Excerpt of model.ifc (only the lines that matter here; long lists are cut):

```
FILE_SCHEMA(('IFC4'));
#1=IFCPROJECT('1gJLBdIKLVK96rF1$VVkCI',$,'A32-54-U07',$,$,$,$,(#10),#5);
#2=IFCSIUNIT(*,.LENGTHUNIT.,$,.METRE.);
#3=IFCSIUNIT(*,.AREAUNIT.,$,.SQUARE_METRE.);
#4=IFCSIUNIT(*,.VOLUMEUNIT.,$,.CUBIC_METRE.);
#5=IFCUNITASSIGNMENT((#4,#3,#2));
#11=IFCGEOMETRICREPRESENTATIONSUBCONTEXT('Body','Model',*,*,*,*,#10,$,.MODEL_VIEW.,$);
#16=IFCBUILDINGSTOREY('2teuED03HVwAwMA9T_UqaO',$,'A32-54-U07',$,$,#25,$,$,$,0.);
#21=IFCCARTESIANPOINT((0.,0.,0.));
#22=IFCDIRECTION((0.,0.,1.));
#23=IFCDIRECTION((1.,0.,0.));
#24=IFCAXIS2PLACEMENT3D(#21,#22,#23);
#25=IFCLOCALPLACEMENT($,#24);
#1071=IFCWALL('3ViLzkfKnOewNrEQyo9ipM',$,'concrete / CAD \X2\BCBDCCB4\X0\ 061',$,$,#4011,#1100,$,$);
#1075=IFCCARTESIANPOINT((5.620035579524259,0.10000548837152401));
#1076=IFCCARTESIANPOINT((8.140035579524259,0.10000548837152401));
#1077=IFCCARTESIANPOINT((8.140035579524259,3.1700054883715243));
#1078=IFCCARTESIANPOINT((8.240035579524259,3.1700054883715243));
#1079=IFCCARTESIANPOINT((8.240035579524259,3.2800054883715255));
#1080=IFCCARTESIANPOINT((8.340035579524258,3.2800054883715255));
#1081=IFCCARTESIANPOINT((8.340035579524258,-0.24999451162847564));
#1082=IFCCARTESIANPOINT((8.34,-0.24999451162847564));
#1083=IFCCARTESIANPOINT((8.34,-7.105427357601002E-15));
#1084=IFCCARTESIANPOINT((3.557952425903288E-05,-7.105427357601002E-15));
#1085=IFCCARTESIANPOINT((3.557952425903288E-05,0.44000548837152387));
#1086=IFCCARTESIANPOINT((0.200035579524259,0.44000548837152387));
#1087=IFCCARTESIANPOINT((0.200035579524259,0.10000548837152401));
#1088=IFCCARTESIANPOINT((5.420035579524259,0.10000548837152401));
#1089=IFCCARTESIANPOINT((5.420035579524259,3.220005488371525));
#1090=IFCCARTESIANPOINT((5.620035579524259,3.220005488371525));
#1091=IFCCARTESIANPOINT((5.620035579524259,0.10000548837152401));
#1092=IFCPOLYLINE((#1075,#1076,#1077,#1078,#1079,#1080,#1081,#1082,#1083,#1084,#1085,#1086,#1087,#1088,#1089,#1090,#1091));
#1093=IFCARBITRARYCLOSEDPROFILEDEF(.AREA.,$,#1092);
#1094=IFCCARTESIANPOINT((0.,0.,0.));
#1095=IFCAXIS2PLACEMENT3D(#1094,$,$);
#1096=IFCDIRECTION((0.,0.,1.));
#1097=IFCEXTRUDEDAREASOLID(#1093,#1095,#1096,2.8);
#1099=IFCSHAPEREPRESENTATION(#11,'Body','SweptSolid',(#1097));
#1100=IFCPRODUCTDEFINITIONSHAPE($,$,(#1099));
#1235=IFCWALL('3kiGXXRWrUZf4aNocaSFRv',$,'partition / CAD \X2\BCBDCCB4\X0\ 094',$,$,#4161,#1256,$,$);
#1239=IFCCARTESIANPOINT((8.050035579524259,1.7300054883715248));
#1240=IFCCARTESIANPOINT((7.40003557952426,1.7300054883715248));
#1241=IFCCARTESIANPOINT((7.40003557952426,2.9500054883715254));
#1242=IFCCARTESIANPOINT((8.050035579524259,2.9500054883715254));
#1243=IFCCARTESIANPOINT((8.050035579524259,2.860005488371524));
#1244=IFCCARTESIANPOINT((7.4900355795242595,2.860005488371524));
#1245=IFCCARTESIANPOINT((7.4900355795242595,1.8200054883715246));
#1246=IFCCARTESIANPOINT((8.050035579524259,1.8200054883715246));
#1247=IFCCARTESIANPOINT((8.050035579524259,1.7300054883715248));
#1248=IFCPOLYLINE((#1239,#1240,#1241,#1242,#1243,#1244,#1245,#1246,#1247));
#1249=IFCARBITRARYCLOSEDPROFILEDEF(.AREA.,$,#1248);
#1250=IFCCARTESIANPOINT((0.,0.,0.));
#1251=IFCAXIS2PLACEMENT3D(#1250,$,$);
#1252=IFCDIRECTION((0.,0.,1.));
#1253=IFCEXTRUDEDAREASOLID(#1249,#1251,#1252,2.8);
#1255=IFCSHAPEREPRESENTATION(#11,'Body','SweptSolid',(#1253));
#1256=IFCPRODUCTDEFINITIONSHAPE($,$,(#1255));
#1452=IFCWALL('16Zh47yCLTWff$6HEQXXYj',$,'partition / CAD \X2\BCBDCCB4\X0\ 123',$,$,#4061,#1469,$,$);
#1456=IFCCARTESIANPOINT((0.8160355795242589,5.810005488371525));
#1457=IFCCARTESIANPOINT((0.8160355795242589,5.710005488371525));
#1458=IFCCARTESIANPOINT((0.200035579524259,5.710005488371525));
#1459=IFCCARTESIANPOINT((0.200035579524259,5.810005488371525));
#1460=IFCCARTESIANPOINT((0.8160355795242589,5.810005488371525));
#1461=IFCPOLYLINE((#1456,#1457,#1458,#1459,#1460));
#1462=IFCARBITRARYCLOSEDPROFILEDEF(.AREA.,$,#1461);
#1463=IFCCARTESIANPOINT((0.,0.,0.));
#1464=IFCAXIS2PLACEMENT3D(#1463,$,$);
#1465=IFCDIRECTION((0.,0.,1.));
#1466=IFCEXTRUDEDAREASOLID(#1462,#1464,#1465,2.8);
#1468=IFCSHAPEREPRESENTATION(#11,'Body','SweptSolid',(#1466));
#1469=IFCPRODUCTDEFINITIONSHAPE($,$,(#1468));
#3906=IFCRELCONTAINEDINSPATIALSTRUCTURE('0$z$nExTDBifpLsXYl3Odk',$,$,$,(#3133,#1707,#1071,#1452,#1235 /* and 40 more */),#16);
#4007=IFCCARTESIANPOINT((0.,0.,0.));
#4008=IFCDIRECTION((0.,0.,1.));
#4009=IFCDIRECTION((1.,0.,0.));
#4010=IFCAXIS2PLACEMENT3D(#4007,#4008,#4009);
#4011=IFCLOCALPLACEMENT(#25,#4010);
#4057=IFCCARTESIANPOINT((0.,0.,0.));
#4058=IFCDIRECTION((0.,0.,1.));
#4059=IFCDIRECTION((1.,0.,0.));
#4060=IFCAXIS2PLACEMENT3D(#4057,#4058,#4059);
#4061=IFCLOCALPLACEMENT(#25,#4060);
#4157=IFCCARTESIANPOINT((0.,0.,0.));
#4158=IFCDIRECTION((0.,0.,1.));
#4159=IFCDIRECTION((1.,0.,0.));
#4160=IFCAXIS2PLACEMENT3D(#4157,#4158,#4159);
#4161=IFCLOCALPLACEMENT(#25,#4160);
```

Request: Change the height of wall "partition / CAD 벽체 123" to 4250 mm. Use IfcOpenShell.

```python
import ifcopenshell
import ifcopenshell.geom
import ifcopenshell.util.representation
import ifcopenshell.util.shape
import ifcopenshell.util.unit

model = ifcopenshell.open("model.ifc")
unit_scale = ifcopenshell.util.unit.calculate_unit_scale(model)
settings = ifcopenshell.geom.settings()


def volume(element):
    """Net volume in cubic metres, openings subtracted."""
    shape = ifcopenshell.geom.create_shape(settings, element)
    return ifcopenshell.util.shape.get_volume(shape.geometry)


wall = model.by_id(1452)
before = volume(wall)

body = ifcopenshell.util.representation.get_representation(wall, "Model", "Body")
solid = body.Items[0]
old_height = solid.Depth
solid.Depth = 4.25 / unit_scale
after = volume(wall)

print(f"height {old_height:g} -> {solid.Depth:g}, volume {before:.3f} -> {after:.3f} m3")

model.write("model-out.ifc")
```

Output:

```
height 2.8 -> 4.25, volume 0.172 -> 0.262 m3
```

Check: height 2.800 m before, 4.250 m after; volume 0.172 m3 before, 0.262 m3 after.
